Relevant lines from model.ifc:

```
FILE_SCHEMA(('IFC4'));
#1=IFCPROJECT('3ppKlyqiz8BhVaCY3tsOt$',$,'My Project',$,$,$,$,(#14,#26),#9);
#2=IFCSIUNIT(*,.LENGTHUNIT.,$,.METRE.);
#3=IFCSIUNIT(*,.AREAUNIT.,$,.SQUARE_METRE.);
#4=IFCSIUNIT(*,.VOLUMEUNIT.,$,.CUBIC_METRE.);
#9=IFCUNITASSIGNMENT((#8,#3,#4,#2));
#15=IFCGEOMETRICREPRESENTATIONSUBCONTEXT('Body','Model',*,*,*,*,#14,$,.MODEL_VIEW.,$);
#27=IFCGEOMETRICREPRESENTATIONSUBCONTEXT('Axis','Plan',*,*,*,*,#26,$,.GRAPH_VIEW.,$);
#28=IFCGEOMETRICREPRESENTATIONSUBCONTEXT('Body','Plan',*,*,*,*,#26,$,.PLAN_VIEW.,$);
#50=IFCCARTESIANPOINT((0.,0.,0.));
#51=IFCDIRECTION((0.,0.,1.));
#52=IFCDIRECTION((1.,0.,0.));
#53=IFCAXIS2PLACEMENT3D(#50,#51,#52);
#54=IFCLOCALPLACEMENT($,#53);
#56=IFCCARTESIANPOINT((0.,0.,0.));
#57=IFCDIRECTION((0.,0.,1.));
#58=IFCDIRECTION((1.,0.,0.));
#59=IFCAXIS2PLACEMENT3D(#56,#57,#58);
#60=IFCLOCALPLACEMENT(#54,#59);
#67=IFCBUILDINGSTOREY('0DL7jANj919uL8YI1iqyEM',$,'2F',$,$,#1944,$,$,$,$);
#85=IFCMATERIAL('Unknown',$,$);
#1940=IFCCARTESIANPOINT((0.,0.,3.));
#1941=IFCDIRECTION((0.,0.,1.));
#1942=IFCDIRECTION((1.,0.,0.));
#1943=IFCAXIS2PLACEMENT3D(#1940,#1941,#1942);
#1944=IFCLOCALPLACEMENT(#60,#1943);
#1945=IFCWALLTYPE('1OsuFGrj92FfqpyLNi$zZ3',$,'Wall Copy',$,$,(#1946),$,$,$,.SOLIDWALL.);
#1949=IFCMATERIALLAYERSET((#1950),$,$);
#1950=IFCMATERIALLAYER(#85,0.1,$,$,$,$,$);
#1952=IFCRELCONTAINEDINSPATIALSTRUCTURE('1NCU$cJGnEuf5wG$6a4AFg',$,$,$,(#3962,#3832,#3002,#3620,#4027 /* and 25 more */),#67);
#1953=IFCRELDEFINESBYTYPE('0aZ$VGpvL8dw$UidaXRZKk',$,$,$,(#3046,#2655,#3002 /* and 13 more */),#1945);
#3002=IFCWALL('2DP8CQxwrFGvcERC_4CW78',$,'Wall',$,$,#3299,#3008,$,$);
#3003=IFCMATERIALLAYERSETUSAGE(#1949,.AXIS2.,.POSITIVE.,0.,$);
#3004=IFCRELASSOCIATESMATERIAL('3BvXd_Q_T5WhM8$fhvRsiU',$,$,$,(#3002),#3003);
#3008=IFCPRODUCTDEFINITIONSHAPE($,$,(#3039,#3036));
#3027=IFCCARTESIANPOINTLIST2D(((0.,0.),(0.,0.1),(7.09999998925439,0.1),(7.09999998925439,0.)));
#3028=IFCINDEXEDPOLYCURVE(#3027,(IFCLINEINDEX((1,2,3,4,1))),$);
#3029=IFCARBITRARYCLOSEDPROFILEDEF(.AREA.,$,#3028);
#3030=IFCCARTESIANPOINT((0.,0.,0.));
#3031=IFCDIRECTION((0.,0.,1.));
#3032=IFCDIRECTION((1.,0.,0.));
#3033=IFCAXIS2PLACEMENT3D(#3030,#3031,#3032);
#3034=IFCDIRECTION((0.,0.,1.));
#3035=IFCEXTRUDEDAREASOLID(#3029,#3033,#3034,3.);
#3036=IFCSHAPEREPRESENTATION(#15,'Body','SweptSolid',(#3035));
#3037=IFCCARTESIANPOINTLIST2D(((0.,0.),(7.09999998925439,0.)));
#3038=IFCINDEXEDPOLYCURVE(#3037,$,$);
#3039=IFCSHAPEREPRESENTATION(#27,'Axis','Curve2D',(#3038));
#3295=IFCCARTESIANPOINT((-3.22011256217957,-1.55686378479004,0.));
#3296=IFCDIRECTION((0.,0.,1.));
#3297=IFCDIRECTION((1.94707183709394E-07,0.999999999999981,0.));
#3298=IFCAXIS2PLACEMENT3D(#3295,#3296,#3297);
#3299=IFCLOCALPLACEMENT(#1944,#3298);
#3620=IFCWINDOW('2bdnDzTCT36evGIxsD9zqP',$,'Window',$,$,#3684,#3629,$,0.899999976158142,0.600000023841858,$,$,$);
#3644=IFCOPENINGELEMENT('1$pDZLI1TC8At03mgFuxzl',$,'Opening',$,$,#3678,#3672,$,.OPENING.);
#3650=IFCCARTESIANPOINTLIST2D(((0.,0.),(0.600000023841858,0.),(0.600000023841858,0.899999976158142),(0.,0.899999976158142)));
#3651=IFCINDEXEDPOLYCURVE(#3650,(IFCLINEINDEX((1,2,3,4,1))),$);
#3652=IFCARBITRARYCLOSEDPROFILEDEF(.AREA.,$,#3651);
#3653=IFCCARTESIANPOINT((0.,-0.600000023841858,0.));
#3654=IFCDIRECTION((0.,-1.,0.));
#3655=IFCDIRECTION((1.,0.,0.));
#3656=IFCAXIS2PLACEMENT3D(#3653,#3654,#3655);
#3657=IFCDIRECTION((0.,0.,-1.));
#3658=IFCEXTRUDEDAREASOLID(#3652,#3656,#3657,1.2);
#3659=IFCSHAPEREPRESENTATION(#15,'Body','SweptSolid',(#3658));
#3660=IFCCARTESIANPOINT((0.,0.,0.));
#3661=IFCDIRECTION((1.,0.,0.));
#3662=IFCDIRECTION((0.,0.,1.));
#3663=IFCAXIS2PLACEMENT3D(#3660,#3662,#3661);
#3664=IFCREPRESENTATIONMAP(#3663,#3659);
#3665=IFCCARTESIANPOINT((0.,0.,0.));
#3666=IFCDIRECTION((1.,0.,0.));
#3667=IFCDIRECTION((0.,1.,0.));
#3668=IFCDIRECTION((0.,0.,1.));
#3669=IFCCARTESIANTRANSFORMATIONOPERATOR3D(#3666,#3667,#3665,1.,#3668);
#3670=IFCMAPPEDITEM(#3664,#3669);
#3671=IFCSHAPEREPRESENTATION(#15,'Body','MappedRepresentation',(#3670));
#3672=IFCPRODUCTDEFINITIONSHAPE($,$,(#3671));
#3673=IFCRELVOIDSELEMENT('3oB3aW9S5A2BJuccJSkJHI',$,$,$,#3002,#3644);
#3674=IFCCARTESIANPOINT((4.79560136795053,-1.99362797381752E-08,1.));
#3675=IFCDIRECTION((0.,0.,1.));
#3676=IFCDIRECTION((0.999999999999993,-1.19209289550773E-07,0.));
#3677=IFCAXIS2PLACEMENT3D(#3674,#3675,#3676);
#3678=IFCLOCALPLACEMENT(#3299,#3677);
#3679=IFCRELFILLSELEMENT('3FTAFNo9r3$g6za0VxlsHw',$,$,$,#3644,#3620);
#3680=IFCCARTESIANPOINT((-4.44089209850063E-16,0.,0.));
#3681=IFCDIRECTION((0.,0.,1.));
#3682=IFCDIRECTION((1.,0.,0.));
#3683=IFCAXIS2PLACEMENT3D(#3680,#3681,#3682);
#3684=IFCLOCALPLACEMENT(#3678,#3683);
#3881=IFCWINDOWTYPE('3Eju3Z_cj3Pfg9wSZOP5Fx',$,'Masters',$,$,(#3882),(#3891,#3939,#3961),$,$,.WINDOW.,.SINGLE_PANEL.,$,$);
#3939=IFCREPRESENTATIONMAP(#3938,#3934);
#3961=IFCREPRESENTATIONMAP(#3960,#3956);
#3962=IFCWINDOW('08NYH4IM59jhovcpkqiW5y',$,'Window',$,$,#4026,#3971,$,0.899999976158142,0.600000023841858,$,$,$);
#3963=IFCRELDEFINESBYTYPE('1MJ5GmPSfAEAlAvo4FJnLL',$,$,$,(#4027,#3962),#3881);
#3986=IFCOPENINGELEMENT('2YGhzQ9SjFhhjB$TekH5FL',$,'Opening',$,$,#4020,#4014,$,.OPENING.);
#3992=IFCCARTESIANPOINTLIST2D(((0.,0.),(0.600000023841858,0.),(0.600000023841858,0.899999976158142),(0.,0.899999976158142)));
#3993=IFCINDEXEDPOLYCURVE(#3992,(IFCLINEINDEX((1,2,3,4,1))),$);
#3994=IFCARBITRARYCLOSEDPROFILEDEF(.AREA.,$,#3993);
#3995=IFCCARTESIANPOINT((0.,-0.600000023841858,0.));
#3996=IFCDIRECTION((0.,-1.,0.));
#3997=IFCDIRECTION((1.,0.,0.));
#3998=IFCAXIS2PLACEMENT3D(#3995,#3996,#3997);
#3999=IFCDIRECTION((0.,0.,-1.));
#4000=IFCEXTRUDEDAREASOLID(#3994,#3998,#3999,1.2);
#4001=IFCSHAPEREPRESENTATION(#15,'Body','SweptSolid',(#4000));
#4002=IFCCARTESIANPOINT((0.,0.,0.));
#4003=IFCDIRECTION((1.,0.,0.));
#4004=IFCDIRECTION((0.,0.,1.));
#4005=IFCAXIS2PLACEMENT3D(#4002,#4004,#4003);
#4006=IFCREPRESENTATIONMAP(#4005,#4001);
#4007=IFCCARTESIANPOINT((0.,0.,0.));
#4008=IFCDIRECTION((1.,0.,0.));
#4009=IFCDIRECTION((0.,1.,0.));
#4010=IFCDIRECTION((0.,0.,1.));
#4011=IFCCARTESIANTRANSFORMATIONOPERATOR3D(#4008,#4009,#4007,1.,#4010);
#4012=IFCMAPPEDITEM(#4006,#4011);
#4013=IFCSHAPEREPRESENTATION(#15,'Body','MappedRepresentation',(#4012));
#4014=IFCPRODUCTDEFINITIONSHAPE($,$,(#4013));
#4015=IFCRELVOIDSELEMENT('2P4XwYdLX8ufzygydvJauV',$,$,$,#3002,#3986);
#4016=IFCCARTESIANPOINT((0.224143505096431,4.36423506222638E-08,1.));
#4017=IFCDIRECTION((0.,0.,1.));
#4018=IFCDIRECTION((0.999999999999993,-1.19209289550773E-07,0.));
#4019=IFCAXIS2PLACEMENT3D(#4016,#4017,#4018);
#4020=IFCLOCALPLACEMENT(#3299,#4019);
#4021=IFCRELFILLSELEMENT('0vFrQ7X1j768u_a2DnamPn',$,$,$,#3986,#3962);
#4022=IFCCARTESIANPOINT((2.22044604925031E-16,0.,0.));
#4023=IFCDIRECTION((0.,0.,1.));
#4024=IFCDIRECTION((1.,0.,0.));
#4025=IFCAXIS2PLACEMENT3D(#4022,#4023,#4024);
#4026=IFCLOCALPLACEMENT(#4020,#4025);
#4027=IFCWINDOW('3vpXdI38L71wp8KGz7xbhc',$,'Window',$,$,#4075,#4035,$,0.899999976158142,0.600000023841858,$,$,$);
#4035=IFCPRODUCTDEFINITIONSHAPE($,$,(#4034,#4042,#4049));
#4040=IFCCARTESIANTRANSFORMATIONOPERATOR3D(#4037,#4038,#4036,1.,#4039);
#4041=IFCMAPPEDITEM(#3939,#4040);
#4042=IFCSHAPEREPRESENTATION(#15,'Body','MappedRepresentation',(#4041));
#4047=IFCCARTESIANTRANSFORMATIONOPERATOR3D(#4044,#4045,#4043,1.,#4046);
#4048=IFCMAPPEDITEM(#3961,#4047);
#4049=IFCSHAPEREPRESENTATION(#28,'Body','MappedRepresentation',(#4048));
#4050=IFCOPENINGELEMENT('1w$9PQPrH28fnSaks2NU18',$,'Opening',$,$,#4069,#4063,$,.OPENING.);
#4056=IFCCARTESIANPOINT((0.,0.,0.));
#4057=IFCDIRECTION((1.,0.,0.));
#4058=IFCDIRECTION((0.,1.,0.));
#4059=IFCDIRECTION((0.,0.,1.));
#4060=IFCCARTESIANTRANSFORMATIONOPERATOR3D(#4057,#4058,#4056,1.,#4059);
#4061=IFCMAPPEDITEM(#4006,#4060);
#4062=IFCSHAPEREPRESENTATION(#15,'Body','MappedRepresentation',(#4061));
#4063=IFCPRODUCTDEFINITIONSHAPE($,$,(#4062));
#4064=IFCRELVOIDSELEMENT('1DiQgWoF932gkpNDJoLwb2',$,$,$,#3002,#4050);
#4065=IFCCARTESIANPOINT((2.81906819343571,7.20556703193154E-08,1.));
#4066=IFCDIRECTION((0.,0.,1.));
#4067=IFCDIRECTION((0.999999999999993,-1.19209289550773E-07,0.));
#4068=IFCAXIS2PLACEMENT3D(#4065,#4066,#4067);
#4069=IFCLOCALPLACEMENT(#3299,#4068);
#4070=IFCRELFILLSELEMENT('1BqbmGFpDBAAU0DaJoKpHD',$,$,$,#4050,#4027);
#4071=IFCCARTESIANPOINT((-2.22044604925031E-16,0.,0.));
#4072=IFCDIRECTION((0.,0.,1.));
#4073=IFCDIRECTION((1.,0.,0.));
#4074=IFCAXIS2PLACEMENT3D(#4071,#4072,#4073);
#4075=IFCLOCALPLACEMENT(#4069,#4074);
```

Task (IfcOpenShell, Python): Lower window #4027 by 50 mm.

```python
import numpy as np
import ifcopenshell
import ifcopenshell.api.geometry
import ifcopenshell.util.placement
import ifcopenshell.util.unit

model = ifcopenshell.open("model.ifc")
unit_scale = ifcopenshell.util.unit.calculate_unit_scale(model)

window = model.by_id(4027)
opening = window.FillsVoids[0].RelatingOpeningElement
dz = -0.05

shift = np.array([0.0, 0.0, dz])
# The window is placed relative to its opening, so it follows when the opening moves.
matrix = ifcopenshell.util.placement.get_local_placement(opening.ObjectPlacement)
matrix[:3, 3] += shift
ifcopenshell.api.geometry.edit_object_placement(
    model, product=opening, matrix=matrix, is_si=False, should_transform_children=True
)

print(f"moved by {dz * unit_scale:+.3f} m")

model.write("model_updated.ifc")
```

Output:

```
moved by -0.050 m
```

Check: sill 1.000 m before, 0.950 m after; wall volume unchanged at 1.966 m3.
